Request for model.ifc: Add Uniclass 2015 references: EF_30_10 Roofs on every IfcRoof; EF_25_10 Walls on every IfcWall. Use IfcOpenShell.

First a look at what the model holds.

```python
import ifcopenshell

model = ifcopenshell.open("model.ifc")
print(model.schema)
print("classifications:", [c.Name for c in model.by_type("IfcClassification")])
for ifc_class in ("IfcDoor", "IfcRoof", "IfcStair", "IfcWall", "IfcWindow"):
    print(ifc_class, len(model.by_type(ifc_class)))
```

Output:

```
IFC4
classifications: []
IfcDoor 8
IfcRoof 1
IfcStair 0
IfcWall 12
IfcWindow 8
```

```python
import ifcopenshell
import ifcopenshell.api.classification

model = ifcopenshell.open("model.ifc")

system = ifcopenshell.api.classification.add_classification(model, classification="Uniclass 2015")

codes = {
    "IfcRoof": ("EF_30_10", "Roofs"),
    "IfcWall": ("EF_25_10", "Walls"),
}
for ifc_class, (code, name) in codes.items():
    products = model.by_type(ifc_class)
    ifcopenshell.api.classification.add_reference(
        model, products=products, classification=system, identification=code, name=name
    )
    print(code, len(products))

model.write("model_rev.ifc")
```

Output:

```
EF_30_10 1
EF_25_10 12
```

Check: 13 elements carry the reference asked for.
